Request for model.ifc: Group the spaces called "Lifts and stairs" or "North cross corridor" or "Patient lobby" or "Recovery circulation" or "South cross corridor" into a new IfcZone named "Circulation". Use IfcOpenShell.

First a look at what the model holds.

```python
import ifcopenshell

model = ifcopenshell.open("model.ifc")
print(model.schema)
seen = {}
for space in model.by_type("IfcSpace"):
    seen[space.Name] = seen.get(space.Name, 0) + 1
for name, count in sorted(seen.items(), key=str):
    print(count, "x", name)
print("zones:", [z.Name for z in model.by_type("IfcZone")][:20])
```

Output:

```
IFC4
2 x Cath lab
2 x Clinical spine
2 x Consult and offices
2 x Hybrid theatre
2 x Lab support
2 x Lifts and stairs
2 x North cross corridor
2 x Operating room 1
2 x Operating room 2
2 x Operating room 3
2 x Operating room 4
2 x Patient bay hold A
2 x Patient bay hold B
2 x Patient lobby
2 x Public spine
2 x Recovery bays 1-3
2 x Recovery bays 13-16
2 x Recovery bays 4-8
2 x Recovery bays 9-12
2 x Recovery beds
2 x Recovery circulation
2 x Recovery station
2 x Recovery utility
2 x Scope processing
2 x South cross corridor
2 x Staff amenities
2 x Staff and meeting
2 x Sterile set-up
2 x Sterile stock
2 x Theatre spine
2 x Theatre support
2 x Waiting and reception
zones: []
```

```python
import ifcopenshell
import ifcopenshell.api.group
import ifcopenshell.api.root

model = ifcopenshell.open("model.ifc")

names = {"Lifts and stairs", "North cross corridor", "Patient lobby", "Recovery circulation", "South cross corridor"}
spaces = [s for s in model.by_type("IfcSpace") if s.Name in names]

zone = ifcopenshell.api.root.create_entity(model, ifc_class="IfcZone", name="Circulation")
ifcopenshell.api.group.assign_group(model, products=spaces, group=zone)
print(len(spaces), "spaces in", zone.Name)

model.write("model-out.ifc")
```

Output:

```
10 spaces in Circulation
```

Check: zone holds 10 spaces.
